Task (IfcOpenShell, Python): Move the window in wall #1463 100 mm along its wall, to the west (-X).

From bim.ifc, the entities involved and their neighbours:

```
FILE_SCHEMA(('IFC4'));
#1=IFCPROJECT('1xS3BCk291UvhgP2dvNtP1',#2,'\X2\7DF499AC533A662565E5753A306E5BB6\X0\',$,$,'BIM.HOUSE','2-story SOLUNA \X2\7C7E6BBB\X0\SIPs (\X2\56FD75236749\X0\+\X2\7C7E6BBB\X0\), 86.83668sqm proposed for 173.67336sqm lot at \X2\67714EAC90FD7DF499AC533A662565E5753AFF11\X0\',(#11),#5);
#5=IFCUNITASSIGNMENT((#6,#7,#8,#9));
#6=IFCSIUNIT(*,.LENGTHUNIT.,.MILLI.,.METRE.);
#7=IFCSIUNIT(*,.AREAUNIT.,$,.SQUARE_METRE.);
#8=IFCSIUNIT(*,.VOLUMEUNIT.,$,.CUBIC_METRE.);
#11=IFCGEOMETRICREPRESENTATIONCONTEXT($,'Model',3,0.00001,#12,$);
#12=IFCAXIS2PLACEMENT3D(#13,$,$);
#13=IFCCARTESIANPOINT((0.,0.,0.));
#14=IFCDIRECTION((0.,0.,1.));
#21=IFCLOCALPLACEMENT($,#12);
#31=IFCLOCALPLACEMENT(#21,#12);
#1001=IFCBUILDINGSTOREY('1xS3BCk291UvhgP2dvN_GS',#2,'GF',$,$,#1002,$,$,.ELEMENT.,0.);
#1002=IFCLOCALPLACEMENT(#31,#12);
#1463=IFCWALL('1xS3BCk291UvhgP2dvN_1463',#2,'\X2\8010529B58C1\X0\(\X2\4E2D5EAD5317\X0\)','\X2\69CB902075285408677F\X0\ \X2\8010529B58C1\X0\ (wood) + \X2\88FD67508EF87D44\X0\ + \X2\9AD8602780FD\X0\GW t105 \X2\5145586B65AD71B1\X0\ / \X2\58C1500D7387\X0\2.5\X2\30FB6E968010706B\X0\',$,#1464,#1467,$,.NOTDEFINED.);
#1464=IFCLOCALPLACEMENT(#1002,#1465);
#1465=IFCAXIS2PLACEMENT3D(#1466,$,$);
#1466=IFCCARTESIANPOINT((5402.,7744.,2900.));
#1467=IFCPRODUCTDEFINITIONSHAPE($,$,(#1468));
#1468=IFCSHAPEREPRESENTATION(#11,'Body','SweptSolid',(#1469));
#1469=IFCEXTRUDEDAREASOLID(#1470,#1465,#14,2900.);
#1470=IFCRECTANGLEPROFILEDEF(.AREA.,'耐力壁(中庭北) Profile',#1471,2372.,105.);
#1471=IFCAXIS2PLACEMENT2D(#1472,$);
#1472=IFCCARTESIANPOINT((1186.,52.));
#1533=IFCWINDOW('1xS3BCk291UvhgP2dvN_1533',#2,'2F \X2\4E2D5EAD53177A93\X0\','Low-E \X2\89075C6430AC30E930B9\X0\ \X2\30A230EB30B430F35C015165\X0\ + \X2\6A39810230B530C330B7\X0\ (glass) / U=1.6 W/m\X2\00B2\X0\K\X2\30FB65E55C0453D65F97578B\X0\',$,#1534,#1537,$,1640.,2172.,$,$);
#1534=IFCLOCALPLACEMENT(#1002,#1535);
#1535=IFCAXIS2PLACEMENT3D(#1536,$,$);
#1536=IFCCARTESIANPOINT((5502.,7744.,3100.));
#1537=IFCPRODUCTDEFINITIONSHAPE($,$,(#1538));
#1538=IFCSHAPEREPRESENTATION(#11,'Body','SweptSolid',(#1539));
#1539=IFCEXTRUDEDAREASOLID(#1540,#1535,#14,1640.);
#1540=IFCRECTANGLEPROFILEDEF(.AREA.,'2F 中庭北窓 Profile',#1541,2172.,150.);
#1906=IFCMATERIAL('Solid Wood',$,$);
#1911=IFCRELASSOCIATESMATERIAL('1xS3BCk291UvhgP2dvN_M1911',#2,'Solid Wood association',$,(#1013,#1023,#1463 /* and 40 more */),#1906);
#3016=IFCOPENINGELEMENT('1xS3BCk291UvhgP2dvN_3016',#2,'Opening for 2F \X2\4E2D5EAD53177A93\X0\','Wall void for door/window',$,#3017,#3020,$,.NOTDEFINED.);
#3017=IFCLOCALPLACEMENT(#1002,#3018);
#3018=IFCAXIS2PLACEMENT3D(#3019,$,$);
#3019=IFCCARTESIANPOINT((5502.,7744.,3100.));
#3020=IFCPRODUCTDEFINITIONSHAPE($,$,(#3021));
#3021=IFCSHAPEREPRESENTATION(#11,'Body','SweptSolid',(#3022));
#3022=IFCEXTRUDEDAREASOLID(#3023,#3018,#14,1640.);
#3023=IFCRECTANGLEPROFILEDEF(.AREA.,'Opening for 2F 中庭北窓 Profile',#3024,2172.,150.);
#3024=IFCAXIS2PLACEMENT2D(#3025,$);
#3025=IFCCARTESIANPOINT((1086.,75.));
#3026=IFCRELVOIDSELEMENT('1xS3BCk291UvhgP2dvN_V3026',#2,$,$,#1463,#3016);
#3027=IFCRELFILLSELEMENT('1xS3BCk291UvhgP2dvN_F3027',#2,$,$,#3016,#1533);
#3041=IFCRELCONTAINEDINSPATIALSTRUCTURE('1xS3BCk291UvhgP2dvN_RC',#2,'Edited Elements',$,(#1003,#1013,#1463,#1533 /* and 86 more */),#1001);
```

```python
import ifcopenshell
import ifcopenshell.api.geometry
import ifcopenshell.util.placement
import ifcopenshell.util.unit

model = ifcopenshell.open("bim.ifc")
unit_scale = ifcopenshell.util.unit.calculate_unit_scale(model)

window = model.by_id(1533)
opening = window.FillsVoids[0].RelatingOpeningElement
wall = opening.VoidsElements[0].RelatingBuildingElement

wall_matrix = ifcopenshell.util.placement.get_local_placement(wall.ObjectPlacement)
shift = wall_matrix[:3, 0] * -0.1 / unit_scale
before = ifcopenshell.util.placement.get_local_placement(window.ObjectPlacement)[:3, 3].copy()

# The window is not placed relative to its opening, so move both.
for product in (opening, window):
    matrix = ifcopenshell.util.placement.get_local_placement(product.ObjectPlacement)
    matrix[:3, 3] += shift
    ifcopenshell.api.geometry.edit_object_placement(model, product=product, matrix=matrix, is_si=False)

after = ifcopenshell.util.placement.get_local_placement(window.ObjectPlacement)[:3, 3]
print("window moved by", (after - before).round(3) + 0.0)

model.write("bim_rev.ifc")
```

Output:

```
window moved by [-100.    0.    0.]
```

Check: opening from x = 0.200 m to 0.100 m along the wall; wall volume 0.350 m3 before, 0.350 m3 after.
